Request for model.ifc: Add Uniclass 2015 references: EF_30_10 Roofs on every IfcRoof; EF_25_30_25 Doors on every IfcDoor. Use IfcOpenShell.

First a look at what the model holds.

```python
import ifcopenshell

model = ifcopenshell.open("model.ifc")
print(model.schema)
print("classifications:", [c.Name for c in model.by_type("IfcClassification")])
for ifc_class in ("IfcDoor", "IfcRoof", "IfcStair", "IfcWall", "IfcWindow"):
    print(ifc_class, len(model.by_type(ifc_class)))
```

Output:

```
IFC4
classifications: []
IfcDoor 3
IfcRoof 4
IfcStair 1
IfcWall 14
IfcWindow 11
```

```python
import ifcopenshell
import ifcopenshell.api.classification

model = ifcopenshell.open("model.ifc")

system = ifcopenshell.api.classification.add_classification(model, classification="Uniclass 2015")

codes = {
    "IfcRoof": ("EF_30_10", "Roofs"),
    "IfcDoor": ("EF_25_30_25", "Doors"),
}
for ifc_class, (code, name) in codes.items():
    products = model.by_type(ifc_class)
    ifcopenshell.api.classification.add_reference(
        model, products=products, classification=system, identification=code, name=name
    )
    print(code, len(products))

model.write("model_edited.ifc")
```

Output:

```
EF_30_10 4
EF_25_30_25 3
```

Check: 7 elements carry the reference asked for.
